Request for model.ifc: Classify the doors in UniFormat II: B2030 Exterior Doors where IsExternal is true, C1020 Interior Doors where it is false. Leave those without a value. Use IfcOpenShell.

First a look at what the model holds.

```python
import ifcopenshell
import ifcopenshell.util.element

model = ifcopenshell.open("model.ifc")
print(model.schema)
print("classifications:", [c.Name for c in model.by_type("IfcClassification")])
values = [ifcopenshell.util.element.get_pset(e, "Pset_DoorCommon", "IsExternal") for e in model.by_type("IfcDoor")]
for value in (True, False, None):
    print("IsExternal", value, values.count(value))
```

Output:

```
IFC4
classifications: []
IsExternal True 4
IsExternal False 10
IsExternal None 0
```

```python
import ifcopenshell
import ifcopenshell.api.classification
import ifcopenshell.util.element

model = ifcopenshell.open("model.ifc")

system = ifcopenshell.api.classification.add_classification(model, classification="UniFormat II")

doors = model.by_type("IfcDoor")
external = {e: ifcopenshell.util.element.get_pset(e, "Pset_DoorCommon", "IsExternal") for e in doors}
for flag, code, name in ((True, "B2030", "Exterior Doors"), (False, "C1020", "Interior Doors")):
    products = [e for e in doors if external[e] is flag]
    ifcopenshell.api.classification.add_reference(
        model, products=products, classification=system, identification=code, name=name
    )
    print(code, len(products))

model.write("model_updated.ifc")
```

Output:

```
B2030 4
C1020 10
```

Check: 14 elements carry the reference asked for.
